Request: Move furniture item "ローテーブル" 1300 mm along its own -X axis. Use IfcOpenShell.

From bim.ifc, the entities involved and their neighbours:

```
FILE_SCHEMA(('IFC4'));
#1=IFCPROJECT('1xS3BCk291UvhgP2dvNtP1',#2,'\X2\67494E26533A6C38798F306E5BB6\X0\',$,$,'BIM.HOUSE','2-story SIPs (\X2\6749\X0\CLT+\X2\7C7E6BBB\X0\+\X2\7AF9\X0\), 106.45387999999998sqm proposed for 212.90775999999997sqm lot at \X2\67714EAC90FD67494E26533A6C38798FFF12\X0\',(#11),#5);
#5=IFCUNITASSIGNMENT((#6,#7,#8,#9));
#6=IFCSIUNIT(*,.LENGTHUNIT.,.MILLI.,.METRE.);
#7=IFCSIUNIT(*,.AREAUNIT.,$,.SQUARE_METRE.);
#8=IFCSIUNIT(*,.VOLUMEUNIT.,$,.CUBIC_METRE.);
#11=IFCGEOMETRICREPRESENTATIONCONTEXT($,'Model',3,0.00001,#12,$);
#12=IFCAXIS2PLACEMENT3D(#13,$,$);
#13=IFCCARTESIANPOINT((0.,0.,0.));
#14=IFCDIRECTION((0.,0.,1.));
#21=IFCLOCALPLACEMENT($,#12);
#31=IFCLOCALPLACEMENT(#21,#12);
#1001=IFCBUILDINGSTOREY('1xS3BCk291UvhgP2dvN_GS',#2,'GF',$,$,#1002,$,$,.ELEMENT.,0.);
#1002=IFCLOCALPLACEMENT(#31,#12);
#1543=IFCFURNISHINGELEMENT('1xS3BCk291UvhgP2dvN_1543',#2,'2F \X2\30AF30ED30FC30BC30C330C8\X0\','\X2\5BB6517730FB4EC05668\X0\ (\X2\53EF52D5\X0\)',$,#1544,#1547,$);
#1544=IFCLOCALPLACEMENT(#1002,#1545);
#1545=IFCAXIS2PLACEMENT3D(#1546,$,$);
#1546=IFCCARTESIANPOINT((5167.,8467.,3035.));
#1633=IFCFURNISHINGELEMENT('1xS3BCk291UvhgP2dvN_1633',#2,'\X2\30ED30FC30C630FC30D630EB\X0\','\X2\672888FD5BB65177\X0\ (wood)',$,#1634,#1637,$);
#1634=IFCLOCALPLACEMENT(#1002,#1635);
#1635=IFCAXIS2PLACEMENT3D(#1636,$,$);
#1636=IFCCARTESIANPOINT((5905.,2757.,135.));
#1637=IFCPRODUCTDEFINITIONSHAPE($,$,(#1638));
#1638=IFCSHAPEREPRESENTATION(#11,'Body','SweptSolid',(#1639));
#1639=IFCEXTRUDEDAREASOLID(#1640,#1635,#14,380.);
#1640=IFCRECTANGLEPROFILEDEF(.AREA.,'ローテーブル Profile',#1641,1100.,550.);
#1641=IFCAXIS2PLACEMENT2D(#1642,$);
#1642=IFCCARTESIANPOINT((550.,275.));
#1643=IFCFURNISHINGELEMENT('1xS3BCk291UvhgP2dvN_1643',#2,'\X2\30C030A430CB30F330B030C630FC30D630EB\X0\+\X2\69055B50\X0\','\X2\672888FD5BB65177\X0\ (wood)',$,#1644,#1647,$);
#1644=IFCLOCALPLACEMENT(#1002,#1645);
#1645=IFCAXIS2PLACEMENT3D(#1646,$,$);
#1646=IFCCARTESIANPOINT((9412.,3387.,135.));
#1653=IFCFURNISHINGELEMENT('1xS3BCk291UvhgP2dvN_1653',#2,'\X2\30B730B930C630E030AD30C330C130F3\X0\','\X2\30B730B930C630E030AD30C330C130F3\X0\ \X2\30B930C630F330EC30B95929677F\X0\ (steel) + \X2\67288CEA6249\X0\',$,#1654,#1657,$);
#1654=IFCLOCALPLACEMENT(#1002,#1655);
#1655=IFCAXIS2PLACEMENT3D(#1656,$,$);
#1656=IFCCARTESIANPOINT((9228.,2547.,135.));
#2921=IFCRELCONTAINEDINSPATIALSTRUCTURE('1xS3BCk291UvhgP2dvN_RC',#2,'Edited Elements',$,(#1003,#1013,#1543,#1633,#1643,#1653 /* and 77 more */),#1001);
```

```python
import ifcopenshell
import ifcopenshell.api.geometry
import ifcopenshell.util.placement

model = ifcopenshell.open("bim.ifc")

item = model.by_guid("1xS3BCk291UvhgP2dvN_1633")
matrix = ifcopenshell.util.placement.get_local_placement(item.ObjectPlacement)
matrix[:3, 3] -= matrix[:3, 0] * 1300.0
ifcopenshell.api.geometry.edit_object_placement(model, product=item, matrix=matrix, is_si=False)

print(ifcopenshell.util.placement.get_local_placement(item.ObjectPlacement).round(3) + 0.0)

model.write("bim_v2.ifc")
```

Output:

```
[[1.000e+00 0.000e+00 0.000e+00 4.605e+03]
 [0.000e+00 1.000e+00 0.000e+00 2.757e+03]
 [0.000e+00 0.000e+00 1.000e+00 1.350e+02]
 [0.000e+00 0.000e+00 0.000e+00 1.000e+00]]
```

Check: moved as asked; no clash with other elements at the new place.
